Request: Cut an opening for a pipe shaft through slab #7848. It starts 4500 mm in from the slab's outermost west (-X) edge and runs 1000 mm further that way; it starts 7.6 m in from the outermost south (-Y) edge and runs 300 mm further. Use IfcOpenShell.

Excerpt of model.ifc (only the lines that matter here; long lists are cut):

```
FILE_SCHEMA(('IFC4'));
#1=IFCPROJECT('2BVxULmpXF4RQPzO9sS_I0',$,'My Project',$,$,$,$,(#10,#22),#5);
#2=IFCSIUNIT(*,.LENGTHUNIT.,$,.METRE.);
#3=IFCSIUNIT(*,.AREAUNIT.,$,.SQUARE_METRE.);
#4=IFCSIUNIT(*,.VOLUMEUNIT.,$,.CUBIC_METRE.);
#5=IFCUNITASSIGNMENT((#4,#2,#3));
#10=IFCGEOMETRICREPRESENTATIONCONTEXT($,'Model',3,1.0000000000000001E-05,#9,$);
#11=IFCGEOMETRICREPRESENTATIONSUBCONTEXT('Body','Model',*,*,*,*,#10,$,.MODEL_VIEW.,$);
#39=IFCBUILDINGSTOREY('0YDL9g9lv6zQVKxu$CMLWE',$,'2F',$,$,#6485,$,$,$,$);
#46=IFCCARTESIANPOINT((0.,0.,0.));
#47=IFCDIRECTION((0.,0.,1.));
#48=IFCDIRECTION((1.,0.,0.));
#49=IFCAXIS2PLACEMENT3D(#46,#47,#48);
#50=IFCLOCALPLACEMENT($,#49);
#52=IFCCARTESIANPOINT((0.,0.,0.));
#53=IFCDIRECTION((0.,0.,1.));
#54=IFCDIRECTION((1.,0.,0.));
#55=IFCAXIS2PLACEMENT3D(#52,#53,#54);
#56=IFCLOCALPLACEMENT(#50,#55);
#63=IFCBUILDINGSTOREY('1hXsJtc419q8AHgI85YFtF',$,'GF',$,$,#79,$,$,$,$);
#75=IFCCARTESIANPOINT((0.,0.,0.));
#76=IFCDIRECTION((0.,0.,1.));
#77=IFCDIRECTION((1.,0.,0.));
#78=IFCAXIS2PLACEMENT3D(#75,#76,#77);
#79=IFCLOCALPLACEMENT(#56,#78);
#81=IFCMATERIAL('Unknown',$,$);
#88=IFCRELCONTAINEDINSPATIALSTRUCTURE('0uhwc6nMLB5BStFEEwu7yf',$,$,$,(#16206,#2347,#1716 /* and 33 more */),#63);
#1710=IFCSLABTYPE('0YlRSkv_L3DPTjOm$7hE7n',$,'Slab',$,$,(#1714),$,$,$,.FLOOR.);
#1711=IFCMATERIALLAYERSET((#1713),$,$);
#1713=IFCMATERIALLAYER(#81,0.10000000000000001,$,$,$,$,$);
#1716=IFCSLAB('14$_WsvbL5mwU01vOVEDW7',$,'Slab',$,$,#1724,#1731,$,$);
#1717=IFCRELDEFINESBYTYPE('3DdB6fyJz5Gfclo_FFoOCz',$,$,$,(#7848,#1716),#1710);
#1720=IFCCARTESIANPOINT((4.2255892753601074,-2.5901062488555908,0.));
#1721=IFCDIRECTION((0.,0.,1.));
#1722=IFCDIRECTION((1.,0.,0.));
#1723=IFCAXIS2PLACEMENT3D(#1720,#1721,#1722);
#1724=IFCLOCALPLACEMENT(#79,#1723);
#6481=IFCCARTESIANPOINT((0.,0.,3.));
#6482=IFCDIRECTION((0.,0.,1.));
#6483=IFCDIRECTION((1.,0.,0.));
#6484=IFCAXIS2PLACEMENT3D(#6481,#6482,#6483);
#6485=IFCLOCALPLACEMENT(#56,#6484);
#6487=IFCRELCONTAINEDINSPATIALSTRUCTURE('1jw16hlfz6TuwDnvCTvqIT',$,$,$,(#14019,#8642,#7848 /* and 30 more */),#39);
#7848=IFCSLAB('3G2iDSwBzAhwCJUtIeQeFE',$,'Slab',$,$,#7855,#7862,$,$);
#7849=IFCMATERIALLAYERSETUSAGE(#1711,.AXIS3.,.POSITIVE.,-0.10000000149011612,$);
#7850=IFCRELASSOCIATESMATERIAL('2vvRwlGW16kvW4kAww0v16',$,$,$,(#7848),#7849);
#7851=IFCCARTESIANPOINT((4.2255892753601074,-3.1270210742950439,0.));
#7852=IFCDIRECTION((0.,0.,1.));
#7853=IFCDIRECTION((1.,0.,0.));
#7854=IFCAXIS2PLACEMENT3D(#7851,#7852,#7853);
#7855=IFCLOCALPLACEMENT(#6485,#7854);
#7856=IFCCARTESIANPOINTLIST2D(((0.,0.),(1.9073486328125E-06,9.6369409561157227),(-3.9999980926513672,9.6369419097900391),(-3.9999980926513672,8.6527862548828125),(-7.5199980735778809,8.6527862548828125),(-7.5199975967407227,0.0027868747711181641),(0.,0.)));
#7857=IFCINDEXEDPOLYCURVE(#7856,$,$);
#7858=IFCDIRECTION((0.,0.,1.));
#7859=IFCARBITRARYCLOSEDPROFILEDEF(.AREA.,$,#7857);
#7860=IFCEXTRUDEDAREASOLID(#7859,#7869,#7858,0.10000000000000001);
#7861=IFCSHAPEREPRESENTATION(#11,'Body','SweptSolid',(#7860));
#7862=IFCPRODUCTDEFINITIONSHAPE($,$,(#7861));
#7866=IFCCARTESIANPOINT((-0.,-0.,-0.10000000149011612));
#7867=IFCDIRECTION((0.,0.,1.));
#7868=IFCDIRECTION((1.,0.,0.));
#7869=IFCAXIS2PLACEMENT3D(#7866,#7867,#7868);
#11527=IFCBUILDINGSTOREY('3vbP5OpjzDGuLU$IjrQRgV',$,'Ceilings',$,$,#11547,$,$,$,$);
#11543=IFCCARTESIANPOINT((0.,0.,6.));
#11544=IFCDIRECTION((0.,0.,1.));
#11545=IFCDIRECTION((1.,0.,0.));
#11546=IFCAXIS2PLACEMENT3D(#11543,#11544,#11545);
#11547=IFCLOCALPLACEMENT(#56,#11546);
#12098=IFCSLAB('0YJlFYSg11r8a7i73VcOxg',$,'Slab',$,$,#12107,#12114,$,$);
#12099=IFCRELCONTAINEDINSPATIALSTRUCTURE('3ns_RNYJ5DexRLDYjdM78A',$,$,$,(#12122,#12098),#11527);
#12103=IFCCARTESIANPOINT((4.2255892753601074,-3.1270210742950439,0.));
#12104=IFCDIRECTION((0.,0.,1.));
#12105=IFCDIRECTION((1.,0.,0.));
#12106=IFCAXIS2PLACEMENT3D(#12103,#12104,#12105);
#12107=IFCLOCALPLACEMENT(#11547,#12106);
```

```python
import numpy as np
import ifcopenshell
import ifcopenshell.api.feature
import ifcopenshell.api.geometry
import ifcopenshell.api.root
import ifcopenshell.geom
import ifcopenshell.util.placement
import ifcopenshell.util.representation
import ifcopenshell.util.shape
import ifcopenshell.util.unit

model = ifcopenshell.open("model.ifc")
unit_scale = ifcopenshell.util.unit.calculate_unit_scale(model)
settings = ifcopenshell.geom.settings()


def volume(element):
    """Net volume in cubic metres, openings subtracted."""
    shape = ifcopenshell.geom.create_shape(settings, element)
    return ifcopenshell.util.shape.get_volume(shape.geometry)


slab = model.by_guid("3G2iDSwBzAhwCJUtIeQeFE")
before = volume(slab)

# Extent in the slab's own axes, in metres. The edges named are its -X and -Y sides.
slab_shape = ifcopenshell.geom.create_shape(settings, slab)
vertices = ifcopenshell.util.shape.get_vertices(slab_shape.geometry)
x_min, y_min, bottom = vertices.min(axis=0)
top = vertices[:, 2].max()

opening = ifcopenshell.api.root.create_entity(model, ifc_class="IfcOpeningElement", name="Pipe shaft opening", predefined_type="OPENING")
context = ifcopenshell.util.representation.get_context(model, "Model", "Body", "MODEL_VIEW")
width, depth = 1, 0.3
outline = [(0.0, 0.0), (width, 0.0), (width, depth), (0.0, depth), (0.0, 0.0)]
# Overshoot both faces by 50 mm so the cut is clean.
shape = ifcopenshell.api.geometry.add_slab_representation(
    model, context=context, depth=top - bottom + 0.1, polyline=outline
)
ifcopenshell.api.geometry.assign_representation(model, product=opening, representation=shape)

matrix = ifcopenshell.util.placement.get_local_placement(slab.ObjectPlacement)
matrix[:, 3] = matrix @ np.append(np.array([x_min + 4.5, y_min + 7.6, bottom - 0.05]) / unit_scale, 1.0)
ifcopenshell.api.geometry.edit_object_placement(model, product=opening, matrix=matrix, is_si=False)
ifcopenshell.api.feature.add_feature(model, feature=opening, element=slab)

after = volume(slab)

print(f"slab volume {before:.3f} -> {after:.3f} m3")

model.write("model-out.ifc")
```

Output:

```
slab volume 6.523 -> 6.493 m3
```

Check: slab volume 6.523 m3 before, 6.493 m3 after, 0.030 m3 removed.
